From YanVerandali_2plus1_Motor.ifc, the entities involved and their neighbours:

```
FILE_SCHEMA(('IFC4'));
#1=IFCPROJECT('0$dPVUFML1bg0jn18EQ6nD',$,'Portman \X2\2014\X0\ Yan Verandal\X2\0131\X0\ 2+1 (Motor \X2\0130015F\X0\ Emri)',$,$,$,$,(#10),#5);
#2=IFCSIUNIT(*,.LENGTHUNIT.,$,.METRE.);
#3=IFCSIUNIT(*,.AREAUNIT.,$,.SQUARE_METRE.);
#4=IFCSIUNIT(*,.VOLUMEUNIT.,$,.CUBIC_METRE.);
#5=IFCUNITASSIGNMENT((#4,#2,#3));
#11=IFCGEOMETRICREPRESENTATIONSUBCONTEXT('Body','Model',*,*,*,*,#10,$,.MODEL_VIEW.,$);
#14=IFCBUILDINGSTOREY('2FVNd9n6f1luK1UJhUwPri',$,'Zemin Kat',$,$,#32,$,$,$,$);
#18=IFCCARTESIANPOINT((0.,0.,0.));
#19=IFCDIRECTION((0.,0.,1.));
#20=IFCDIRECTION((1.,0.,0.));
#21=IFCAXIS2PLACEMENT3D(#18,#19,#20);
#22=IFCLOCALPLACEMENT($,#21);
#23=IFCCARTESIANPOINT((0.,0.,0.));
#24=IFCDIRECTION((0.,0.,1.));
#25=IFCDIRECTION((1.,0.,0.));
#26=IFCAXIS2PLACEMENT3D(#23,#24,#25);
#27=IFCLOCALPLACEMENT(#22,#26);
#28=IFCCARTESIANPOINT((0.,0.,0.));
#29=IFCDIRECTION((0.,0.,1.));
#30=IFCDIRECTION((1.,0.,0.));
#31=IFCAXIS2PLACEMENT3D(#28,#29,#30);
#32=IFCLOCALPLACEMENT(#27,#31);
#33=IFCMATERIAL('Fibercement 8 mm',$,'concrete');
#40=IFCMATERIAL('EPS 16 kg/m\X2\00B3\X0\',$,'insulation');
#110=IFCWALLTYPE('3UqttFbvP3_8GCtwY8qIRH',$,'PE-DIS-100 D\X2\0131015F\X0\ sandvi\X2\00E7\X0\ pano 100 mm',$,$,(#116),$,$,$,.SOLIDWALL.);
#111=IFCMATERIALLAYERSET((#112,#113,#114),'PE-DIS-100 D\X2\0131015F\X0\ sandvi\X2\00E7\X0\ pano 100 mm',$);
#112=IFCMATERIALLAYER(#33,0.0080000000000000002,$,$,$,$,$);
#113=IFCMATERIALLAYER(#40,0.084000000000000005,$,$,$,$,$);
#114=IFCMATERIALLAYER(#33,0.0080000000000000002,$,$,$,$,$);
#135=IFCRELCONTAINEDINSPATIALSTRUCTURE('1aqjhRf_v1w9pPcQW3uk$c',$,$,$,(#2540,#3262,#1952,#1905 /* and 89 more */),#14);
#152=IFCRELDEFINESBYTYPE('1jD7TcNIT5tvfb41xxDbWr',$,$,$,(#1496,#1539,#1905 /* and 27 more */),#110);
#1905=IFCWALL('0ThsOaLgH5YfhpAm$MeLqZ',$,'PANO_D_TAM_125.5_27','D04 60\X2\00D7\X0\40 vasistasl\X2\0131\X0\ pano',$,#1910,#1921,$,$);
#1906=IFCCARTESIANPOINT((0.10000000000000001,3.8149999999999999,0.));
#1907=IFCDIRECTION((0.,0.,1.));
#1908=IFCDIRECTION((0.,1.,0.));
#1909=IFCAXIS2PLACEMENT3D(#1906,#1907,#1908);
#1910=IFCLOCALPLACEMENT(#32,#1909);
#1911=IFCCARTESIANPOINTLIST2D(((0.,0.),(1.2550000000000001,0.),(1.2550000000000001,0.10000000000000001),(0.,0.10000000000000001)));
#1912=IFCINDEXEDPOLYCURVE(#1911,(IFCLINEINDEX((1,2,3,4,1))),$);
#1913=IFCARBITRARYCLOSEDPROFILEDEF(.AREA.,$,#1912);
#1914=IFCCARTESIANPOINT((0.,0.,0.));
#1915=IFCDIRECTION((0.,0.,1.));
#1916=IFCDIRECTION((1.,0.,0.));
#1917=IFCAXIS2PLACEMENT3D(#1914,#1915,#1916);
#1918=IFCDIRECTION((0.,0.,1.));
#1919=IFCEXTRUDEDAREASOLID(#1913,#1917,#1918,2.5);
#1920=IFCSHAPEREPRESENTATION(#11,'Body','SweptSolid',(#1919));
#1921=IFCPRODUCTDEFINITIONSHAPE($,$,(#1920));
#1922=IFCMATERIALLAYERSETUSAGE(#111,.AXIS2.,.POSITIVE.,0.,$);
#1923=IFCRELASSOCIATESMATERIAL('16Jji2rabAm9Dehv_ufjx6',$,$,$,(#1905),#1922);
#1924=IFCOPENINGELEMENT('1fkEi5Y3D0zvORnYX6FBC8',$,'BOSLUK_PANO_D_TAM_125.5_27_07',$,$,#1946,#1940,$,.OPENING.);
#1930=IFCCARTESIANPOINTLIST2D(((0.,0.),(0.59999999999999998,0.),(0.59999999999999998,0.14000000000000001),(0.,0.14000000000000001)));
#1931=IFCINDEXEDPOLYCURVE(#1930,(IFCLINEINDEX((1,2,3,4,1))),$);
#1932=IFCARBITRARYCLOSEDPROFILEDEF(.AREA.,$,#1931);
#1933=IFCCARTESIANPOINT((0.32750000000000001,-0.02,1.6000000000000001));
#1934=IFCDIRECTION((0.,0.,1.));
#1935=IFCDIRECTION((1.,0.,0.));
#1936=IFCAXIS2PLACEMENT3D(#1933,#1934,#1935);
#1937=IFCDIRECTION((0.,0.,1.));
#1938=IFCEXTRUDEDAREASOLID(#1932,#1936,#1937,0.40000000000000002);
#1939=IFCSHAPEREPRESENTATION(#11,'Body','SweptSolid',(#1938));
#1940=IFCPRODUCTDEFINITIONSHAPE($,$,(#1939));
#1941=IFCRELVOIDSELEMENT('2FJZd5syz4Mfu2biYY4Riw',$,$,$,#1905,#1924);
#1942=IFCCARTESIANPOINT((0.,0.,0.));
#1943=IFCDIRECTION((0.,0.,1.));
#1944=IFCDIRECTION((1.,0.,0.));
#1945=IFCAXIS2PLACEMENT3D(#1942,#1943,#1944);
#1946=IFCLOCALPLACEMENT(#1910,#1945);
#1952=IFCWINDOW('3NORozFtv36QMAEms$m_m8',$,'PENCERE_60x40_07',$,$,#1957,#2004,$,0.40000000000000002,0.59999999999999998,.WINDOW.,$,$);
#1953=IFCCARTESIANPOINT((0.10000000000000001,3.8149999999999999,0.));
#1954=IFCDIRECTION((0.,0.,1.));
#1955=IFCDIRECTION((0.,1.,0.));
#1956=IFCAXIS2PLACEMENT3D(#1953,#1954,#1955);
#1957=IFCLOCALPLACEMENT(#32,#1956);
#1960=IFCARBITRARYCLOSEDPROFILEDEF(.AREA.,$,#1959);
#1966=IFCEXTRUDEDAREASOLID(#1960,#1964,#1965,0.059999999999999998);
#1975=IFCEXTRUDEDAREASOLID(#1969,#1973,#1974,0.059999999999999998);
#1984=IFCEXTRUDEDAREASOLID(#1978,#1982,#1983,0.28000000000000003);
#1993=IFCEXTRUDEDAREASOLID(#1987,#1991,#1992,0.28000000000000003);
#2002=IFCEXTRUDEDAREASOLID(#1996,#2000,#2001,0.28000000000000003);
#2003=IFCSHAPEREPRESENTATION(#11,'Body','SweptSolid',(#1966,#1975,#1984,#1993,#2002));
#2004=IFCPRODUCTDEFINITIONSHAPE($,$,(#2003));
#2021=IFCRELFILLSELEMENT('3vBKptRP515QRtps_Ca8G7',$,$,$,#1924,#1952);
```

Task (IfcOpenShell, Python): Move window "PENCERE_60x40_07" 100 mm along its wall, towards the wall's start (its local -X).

```python
import ifcopenshell
import ifcopenshell.api.geometry
import ifcopenshell.util.placement
import ifcopenshell.util.unit

model = ifcopenshell.open("YanVerandali_2plus1_Motor.ifc")
unit_scale = ifcopenshell.util.unit.calculate_unit_scale(model)

window = model.by_guid("3NORozFtv36QMAEms$m_m8")
opening = window.FillsVoids[0].RelatingOpeningElement
wall = opening.VoidsElements[0].RelatingBuildingElement

wall_matrix = ifcopenshell.util.placement.get_local_placement(wall.ObjectPlacement)
shift = wall_matrix[:3, 0] * -0.1 / unit_scale
before = ifcopenshell.util.placement.get_local_placement(window.ObjectPlacement)[:3, 3].copy()

# The window is not placed relative to its opening, so move both.
for product in (opening, window):
    matrix = ifcopenshell.util.placement.get_local_placement(product.ObjectPlacement)
    matrix[:3, 3] += shift
    ifcopenshell.api.geometry.edit_object_placement(model, product=product, matrix=matrix, is_si=False)

after = ifcopenshell.util.placement.get_local_placement(window.ObjectPlacement)[:3, 3]
print("window moved by", (after - before).round(3) + 0.0)

model.write("YanVerandali_2plus1_Motor_v2.ifc")
```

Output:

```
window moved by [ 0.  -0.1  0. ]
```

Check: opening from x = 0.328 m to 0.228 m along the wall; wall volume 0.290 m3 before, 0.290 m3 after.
